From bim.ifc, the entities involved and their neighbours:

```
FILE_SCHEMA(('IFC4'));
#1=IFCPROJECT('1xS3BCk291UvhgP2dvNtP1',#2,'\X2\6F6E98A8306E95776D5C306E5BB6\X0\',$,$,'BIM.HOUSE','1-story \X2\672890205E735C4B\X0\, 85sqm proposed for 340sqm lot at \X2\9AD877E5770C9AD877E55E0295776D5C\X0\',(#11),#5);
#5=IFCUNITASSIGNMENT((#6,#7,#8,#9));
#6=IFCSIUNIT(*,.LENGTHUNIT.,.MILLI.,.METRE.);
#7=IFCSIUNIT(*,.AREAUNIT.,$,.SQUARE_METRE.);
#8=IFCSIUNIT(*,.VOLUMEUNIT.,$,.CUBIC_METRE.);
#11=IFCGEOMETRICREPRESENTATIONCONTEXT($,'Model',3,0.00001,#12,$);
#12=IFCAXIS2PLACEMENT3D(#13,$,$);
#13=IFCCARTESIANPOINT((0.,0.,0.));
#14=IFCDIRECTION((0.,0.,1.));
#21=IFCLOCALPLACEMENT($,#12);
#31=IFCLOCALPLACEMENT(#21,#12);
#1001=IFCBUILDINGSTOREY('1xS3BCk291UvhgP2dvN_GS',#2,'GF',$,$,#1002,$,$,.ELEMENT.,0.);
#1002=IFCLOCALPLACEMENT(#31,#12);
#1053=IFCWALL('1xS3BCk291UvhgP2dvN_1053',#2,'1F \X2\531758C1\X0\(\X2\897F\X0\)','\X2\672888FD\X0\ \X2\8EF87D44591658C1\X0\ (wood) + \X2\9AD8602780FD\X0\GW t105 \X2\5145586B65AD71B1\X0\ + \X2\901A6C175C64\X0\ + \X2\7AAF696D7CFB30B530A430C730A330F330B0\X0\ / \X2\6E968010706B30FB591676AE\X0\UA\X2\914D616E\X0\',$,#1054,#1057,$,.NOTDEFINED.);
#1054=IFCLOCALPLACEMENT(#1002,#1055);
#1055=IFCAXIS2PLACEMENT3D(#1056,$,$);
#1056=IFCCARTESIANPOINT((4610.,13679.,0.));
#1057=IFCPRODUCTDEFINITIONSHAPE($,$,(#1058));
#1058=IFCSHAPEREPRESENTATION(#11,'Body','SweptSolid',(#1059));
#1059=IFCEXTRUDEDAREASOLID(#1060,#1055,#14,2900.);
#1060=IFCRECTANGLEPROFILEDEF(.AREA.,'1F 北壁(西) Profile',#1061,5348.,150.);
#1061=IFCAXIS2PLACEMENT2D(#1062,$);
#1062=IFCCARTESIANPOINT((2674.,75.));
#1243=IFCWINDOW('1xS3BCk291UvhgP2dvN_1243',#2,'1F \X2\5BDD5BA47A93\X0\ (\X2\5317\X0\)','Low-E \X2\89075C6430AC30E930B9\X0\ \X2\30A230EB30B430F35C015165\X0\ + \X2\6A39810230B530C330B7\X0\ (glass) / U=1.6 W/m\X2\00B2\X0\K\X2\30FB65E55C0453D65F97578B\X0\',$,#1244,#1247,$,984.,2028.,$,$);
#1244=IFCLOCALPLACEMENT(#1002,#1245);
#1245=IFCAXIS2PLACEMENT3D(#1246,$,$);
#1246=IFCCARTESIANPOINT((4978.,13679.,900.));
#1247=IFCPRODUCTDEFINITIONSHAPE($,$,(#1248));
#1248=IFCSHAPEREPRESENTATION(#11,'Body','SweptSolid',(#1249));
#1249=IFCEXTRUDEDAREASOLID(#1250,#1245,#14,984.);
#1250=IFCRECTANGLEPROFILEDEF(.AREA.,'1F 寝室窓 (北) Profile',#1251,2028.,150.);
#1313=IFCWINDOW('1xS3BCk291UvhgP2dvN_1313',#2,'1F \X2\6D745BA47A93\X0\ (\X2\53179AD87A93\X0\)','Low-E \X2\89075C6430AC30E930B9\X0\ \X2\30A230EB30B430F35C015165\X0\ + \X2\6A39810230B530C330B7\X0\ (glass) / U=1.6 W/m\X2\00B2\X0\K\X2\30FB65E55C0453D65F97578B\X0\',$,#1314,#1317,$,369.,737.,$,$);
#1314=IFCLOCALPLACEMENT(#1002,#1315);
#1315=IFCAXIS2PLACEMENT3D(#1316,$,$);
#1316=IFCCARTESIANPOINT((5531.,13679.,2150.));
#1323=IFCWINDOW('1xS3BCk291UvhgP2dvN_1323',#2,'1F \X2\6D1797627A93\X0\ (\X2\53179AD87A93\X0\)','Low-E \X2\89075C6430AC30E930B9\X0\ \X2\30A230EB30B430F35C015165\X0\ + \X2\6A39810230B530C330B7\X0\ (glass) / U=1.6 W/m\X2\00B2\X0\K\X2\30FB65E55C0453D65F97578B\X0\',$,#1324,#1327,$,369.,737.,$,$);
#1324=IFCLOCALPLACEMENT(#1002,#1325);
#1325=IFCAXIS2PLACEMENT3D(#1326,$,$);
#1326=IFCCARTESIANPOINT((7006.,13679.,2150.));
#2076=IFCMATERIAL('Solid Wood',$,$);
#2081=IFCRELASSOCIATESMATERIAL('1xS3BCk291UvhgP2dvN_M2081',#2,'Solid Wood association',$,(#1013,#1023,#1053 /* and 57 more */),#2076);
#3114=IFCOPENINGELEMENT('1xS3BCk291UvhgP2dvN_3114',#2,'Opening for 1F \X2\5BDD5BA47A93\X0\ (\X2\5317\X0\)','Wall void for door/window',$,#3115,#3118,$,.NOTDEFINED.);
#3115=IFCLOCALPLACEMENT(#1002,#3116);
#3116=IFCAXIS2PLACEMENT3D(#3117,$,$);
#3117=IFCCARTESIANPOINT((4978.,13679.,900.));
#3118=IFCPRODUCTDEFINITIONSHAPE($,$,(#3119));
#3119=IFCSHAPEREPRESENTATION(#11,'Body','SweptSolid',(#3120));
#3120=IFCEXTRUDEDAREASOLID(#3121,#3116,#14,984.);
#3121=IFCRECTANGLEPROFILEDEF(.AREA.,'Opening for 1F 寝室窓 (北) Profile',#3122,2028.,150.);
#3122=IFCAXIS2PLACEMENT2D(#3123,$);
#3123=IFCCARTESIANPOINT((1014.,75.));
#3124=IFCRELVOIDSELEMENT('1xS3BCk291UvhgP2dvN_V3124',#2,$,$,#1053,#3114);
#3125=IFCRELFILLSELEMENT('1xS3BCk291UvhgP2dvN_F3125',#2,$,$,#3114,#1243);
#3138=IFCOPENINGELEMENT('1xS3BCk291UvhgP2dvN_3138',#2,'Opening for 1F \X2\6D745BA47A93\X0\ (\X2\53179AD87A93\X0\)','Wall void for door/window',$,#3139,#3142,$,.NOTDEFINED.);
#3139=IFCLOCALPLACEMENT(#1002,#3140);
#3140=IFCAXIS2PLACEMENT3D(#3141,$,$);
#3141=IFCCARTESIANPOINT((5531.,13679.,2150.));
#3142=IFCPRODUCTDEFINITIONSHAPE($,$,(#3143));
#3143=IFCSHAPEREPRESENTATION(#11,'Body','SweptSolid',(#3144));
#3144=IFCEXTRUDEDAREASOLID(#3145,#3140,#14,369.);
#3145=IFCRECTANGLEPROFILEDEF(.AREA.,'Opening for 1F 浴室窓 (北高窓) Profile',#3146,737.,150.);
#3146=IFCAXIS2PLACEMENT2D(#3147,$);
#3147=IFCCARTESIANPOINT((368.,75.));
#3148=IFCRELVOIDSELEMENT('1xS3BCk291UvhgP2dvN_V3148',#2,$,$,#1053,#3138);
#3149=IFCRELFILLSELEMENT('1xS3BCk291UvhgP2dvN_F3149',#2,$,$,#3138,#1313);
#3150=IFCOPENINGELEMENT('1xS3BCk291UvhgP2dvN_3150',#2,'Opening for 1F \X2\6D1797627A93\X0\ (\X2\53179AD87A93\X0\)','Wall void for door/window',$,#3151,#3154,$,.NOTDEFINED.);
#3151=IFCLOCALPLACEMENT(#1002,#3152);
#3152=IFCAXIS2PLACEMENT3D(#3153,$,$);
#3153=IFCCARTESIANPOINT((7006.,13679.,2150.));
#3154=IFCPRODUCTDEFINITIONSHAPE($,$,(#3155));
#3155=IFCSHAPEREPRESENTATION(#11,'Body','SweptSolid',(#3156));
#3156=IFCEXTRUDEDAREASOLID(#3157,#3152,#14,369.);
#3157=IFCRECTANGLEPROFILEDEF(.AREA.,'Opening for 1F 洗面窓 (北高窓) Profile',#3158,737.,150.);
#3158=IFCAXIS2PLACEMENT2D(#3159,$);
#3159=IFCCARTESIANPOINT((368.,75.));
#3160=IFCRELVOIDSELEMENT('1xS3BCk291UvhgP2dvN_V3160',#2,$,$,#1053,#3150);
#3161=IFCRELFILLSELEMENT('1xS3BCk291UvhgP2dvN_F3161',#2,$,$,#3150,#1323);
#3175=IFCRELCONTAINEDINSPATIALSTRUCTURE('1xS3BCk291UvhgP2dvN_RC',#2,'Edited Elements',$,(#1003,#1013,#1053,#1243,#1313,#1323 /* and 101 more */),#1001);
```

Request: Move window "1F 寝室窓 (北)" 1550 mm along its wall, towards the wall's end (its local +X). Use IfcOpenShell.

```python
import ifcopenshell
import ifcopenshell.api.geometry
import ifcopenshell.util.placement
import ifcopenshell.util.unit

model = ifcopenshell.open("bim.ifc")
unit_scale = ifcopenshell.util.unit.calculate_unit_scale(model)

window = model.by_guid("1xS3BCk291UvhgP2dvN_1243")
opening = window.FillsVoids[0].RelatingOpeningElement
wall = opening.VoidsElements[0].RelatingBuildingElement

wall_matrix = ifcopenshell.util.placement.get_local_placement(wall.ObjectPlacement)
shift = wall_matrix[:3, 0] * 1.55 / unit_scale
before = ifcopenshell.util.placement.get_local_placement(window.ObjectPlacement)[:3, 3].copy()

# The window is not placed relative to its opening, so move both.
for product in (opening, window):
    matrix = ifcopenshell.util.placement.get_local_placement(product.ObjectPlacement)
    matrix[:3, 3] += shift
    ifcopenshell.api.geometry.edit_object_placement(model, product=product, matrix=matrix, is_si=False)

after = ifcopenshell.util.placement.get_local_placement(window.ObjectPlacement)[:3, 3]
print("window moved by", (after - before).round(3) + 0.0)

model.write("bim_updated.ifc")
```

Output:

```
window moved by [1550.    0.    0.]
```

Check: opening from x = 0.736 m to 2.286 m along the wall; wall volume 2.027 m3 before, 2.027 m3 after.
